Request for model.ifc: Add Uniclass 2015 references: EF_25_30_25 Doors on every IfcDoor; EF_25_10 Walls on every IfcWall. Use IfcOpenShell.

First a look at what the model holds.

```python
import ifcopenshell

model = ifcopenshell.open("model.ifc")
print(model.schema)
print("classifications:", [c.Name for c in model.by_type("IfcClassification")])
for ifc_class in ("IfcDoor", "IfcRoof", "IfcStair", "IfcWall", "IfcWindow"):
    print(ifc_class, len(model.by_type(ifc_class)))
```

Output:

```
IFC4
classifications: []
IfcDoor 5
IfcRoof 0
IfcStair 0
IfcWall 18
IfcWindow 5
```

```python
import ifcopenshell
import ifcopenshell.api.classification

model = ifcopenshell.open("model.ifc")

system = ifcopenshell.api.classification.add_classification(model, classification="Uniclass 2015")

codes = {
    "IfcDoor": ("EF_25_30_25", "Doors"),
    "IfcWall": ("EF_25_10", "Walls"),
}
for ifc_class, (code, name) in codes.items():
    products = model.by_type(ifc_class)
    ifcopenshell.api.classification.add_reference(
        model, products=products, classification=system, identification=code, name=name
    )
    print(code, len(products))

model.write("model_edited.ifc")
```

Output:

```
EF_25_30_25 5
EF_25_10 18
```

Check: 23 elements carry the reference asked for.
